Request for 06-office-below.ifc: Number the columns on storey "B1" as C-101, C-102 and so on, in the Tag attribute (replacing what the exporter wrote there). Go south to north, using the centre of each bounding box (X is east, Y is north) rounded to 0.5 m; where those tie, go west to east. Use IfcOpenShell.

First a look at what the model holds.

```python
import ifcopenshell
import ifcopenshell.util.element
import ifcopenshell.util.placement

model = ifcopenshell.open("06-office-below.ifc")
print(model.schema)
storey = next(s for s in model.by_type("IfcBuildingStorey") if s.Name == "B1")
columns = [e for e in ifcopenshell.util.element.get_decomposition(storey) if e.is_a("IfcColumn")]
for e in sorted(columns, key=lambda e: e.id()):
    origin = ifcopenshell.util.placement.get_local_placement(e.ObjectPlacement)[:3, 3]
    print(e.id(), e.Tag, e.Name, origin.round(2) + 0.0, sep=" | ")
```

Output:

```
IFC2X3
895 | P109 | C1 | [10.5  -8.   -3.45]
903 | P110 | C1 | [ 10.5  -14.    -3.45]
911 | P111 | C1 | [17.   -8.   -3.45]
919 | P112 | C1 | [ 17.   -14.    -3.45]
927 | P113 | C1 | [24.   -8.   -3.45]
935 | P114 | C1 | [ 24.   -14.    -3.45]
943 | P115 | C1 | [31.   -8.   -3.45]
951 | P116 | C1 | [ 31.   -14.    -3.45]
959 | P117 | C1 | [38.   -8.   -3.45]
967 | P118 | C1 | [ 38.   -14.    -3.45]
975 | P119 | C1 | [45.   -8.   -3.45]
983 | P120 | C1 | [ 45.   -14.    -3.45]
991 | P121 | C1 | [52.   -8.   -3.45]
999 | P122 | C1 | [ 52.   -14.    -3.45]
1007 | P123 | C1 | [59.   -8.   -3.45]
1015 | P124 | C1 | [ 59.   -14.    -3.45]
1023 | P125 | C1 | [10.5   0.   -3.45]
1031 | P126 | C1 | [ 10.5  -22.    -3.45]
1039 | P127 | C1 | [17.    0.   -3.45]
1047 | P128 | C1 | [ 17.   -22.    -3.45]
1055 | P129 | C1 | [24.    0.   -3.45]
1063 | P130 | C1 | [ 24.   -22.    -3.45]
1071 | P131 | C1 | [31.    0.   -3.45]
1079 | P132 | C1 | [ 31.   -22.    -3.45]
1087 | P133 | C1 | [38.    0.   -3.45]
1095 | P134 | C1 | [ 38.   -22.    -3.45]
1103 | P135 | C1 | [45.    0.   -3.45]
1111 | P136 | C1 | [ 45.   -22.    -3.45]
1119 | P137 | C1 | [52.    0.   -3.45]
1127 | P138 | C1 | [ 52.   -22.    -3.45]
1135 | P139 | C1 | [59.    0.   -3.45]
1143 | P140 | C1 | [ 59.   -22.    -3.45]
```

```python
import ifcopenshell
import ifcopenshell.geom
import ifcopenshell.util.element
import ifcopenshell.util.shape

model = ifcopenshell.open("06-office-below.ifc")
settings = ifcopenshell.geom.settings()
settings.set("use-world-coords", True)


def centre(element):
    shape = ifcopenshell.geom.create_shape(settings, element)
    return ifcopenshell.util.shape.get_bbox_centroid(shape.geometry)


storey = next(s for s in model.by_type("IfcBuildingStorey") if s.Name == "B1")
columns = [e for e in ifcopenshell.util.element.get_decomposition(storey) if e.is_a("IfcColumn")]

# Insertion points can sit at a corner or the storey origin, so sort by the geometry (in metres).
centres = {e: centre(e) for e in columns}
columns.sort(key=lambda e: (round(centres[e][1] / 0.5), centres[e][0]))

for i, e in enumerate(columns, start=1):
    number = f"C-1{i:02d}"
    e.Tag = number
    print(e.id(), number)

model.write("06-office-below_edited.ifc")
```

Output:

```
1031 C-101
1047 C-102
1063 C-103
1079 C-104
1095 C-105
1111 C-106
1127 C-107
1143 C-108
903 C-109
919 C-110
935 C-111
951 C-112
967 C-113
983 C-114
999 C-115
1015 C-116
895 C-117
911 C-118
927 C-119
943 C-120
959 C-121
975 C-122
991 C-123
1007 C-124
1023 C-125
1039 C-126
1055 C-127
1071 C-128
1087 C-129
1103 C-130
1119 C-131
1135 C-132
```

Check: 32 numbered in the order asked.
